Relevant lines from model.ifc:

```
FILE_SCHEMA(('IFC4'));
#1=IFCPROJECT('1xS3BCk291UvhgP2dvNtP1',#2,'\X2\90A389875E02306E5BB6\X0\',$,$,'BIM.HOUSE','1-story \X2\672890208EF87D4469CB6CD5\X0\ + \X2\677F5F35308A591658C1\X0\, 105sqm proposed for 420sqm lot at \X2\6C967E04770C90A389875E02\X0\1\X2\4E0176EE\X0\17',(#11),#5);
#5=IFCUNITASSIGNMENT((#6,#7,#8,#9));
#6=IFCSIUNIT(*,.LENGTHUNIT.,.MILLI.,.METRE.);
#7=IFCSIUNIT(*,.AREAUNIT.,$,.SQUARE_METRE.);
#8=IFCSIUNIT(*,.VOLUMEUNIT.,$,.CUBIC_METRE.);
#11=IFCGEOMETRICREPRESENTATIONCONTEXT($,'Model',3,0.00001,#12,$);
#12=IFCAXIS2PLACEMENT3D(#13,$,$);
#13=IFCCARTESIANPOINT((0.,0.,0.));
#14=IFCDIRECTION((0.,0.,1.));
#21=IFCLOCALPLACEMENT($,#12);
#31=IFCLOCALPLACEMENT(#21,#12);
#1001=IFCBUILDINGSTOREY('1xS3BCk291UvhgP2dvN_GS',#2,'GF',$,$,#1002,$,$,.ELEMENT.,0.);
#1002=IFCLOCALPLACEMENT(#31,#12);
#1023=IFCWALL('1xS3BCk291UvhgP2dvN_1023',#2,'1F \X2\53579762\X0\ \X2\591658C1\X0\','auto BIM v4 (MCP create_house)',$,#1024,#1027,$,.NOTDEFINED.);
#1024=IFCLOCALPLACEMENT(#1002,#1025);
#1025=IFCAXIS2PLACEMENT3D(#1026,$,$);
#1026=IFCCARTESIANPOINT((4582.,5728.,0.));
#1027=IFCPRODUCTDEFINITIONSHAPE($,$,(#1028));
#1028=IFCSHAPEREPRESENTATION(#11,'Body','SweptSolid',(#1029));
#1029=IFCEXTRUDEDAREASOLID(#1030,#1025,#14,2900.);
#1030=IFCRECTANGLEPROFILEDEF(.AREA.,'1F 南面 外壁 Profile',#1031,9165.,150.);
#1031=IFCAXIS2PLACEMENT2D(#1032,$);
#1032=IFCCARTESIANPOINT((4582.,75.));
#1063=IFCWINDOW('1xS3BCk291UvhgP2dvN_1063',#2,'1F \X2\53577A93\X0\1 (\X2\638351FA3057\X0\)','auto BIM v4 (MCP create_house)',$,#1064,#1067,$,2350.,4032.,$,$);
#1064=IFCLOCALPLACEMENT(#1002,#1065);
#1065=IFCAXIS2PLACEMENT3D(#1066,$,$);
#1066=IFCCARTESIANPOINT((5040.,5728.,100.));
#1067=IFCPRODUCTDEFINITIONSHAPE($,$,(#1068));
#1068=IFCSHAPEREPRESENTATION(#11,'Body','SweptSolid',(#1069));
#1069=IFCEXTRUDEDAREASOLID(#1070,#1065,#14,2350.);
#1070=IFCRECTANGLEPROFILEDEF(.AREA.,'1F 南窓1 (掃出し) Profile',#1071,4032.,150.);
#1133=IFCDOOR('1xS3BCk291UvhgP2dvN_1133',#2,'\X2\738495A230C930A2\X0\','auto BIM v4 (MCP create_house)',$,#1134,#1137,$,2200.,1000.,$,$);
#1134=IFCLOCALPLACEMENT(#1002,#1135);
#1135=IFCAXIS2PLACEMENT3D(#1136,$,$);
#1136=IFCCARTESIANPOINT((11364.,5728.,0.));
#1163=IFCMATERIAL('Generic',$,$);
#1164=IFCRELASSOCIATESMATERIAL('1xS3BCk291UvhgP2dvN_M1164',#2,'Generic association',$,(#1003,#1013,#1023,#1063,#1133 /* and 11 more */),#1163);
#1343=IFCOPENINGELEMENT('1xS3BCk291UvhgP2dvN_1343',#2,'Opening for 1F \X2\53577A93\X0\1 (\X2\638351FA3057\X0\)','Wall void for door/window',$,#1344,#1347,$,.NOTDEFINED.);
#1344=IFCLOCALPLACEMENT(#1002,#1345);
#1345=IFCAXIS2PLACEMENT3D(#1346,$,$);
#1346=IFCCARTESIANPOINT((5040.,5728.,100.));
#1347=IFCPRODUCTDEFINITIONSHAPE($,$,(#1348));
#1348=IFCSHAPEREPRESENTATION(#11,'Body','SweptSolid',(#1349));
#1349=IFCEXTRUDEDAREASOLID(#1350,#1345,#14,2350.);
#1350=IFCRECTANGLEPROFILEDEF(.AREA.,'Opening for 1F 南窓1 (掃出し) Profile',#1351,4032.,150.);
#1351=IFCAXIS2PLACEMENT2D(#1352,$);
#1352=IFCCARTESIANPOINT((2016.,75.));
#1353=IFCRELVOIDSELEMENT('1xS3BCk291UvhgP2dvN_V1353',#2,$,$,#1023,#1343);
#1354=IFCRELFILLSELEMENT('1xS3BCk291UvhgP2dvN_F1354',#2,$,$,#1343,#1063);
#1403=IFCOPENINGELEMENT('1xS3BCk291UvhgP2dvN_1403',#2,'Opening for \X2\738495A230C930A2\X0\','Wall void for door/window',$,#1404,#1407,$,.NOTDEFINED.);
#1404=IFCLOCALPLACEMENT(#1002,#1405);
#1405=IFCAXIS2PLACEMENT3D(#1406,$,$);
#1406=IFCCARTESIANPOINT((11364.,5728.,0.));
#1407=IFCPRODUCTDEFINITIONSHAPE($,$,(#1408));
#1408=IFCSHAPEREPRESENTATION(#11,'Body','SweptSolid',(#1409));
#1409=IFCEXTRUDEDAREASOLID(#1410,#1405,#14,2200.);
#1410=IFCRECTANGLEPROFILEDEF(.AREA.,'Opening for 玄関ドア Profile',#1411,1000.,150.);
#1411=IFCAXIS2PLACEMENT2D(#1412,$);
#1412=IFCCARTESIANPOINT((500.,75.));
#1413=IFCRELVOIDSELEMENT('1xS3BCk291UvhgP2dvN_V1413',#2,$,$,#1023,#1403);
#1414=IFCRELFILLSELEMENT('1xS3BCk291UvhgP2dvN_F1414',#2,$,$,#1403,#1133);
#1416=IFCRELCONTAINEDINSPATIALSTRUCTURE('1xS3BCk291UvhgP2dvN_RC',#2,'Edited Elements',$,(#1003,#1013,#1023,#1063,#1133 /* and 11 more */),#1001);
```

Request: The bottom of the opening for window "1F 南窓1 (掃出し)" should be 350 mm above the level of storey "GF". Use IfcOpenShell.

```python
import numpy as np
import ifcopenshell
import ifcopenshell.api.geometry
import ifcopenshell.geom
import ifcopenshell.util.element
import ifcopenshell.util.placement
import ifcopenshell.util.shape
import ifcopenshell.util.unit

model = ifcopenshell.open("model.ifc")
unit_scale = ifcopenshell.util.unit.calculate_unit_scale(model)

window = model.by_guid("1xS3BCk291UvhgP2dvN_1063")
opening = window.FillsVoids[0].RelatingOpeningElement
storey = ifcopenshell.util.element.get_container(window, ifc_class="IfcBuildingStorey")
level = ifcopenshell.util.placement.get_local_placement(storey.ObjectPlacement)[2, 3]

# The opening's origin need not be at the sill, so measure its lowest point.
shape = ifcopenshell.geom.create_shape(ifcopenshell.geom.settings(), opening)
bottom = ifcopenshell.util.shape.get_shape_bottom_elevation(shape, shape.geometry) / unit_scale
dz = level + 350.0 - bottom

shift = np.array([0.0, 0.0, dz])
# The window is not placed relative to its opening, so move both.
for product in (opening, window):
    matrix = ifcopenshell.util.placement.get_local_placement(product.ObjectPlacement)
    matrix[:3, 3] += shift
    ifcopenshell.api.geometry.edit_object_placement(model, product=product, matrix=matrix, is_si=False)

print(f"moved by {dz * unit_scale:+.3f} m")

model.write("model-out.ifc")
```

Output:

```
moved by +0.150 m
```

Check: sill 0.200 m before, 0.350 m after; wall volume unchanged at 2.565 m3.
